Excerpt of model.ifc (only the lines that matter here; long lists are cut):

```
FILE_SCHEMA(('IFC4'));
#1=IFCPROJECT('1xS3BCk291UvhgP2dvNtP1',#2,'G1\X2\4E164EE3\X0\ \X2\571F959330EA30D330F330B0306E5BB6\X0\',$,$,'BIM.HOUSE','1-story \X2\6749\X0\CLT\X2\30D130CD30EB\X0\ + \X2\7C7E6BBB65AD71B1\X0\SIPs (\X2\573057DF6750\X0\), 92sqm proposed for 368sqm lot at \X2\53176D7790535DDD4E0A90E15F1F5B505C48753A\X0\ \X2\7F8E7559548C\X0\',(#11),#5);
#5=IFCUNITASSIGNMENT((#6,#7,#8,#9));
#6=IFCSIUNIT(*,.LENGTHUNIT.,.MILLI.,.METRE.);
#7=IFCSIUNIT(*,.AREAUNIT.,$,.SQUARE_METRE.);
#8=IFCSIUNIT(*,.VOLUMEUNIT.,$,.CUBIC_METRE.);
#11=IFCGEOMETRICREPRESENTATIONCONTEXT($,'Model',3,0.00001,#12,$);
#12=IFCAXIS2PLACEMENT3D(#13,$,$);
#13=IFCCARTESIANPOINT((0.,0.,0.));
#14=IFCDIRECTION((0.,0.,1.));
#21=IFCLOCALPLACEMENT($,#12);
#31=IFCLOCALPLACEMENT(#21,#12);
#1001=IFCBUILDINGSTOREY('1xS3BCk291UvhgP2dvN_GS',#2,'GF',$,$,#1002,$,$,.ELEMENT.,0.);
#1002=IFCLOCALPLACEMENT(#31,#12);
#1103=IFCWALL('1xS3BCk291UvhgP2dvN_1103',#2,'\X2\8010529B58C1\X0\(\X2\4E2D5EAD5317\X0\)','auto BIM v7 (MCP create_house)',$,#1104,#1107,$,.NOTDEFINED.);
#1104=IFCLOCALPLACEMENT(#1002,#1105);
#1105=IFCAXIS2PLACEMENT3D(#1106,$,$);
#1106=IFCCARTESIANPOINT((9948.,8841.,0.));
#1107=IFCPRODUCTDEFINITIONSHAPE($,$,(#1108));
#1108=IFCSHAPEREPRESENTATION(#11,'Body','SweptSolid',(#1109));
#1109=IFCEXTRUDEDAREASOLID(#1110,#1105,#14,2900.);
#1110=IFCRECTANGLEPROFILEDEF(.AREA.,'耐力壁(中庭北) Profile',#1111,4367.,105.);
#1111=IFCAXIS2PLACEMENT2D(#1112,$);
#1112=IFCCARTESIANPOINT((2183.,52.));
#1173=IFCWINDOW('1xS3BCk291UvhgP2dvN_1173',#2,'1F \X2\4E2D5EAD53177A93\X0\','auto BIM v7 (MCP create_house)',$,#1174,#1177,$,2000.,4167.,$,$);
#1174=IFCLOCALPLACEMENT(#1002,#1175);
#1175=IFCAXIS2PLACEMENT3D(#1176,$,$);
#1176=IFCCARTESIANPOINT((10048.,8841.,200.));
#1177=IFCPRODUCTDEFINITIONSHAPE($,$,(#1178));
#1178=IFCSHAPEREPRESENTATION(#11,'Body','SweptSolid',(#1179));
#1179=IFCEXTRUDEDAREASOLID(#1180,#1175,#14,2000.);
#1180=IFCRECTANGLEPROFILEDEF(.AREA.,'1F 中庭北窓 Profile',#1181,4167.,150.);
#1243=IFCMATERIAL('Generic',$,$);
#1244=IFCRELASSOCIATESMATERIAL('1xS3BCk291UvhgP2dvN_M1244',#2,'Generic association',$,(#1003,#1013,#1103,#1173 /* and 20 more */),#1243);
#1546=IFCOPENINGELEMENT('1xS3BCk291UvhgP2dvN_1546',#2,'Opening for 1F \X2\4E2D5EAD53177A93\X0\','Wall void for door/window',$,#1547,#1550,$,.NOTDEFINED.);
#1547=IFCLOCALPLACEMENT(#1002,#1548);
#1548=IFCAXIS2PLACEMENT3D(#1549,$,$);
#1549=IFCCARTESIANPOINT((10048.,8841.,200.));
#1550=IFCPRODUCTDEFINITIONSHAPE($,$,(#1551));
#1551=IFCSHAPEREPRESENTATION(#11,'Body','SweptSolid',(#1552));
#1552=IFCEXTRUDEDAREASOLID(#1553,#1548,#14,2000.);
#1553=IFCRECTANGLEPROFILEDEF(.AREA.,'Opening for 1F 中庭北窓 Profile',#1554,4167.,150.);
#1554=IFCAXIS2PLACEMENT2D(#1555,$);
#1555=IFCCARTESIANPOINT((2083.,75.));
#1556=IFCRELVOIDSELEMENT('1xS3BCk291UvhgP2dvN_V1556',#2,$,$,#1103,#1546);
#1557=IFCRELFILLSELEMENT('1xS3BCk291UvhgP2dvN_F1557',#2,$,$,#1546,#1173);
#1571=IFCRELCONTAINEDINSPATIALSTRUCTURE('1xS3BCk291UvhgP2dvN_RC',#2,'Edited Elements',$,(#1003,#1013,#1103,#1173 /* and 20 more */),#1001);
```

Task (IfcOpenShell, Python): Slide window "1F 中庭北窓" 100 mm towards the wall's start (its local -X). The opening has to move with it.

```python
import ifcopenshell
import ifcopenshell.api.geometry
import ifcopenshell.util.placement
import ifcopenshell.util.unit

model = ifcopenshell.open("model.ifc")
unit_scale = ifcopenshell.util.unit.calculate_unit_scale(model)

window = model.by_guid("1xS3BCk291UvhgP2dvN_1173")
opening = window.FillsVoids[0].RelatingOpeningElement
wall = opening.VoidsElements[0].RelatingBuildingElement

wall_matrix = ifcopenshell.util.placement.get_local_placement(wall.ObjectPlacement)
shift = wall_matrix[:3, 0] * -0.1 / unit_scale
before = ifcopenshell.util.placement.get_local_placement(window.ObjectPlacement)[:3, 3].copy()

# The window is not placed relative to its opening, so move both.
for product in (opening, window):
    matrix = ifcopenshell.util.placement.get_local_placement(product.ObjectPlacement)
    matrix[:3, 3] += shift
    ifcopenshell.api.geometry.edit_object_placement(model, product=product, matrix=matrix, is_si=False)

after = ifcopenshell.util.placement.get_local_placement(window.ObjectPlacement)[:3, 3]
print("window moved by", (after - before).round(3) + 0.0)

model.write("model_updated.ifc")
```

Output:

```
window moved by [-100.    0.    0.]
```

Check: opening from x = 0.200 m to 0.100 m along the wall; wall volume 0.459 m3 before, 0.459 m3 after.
